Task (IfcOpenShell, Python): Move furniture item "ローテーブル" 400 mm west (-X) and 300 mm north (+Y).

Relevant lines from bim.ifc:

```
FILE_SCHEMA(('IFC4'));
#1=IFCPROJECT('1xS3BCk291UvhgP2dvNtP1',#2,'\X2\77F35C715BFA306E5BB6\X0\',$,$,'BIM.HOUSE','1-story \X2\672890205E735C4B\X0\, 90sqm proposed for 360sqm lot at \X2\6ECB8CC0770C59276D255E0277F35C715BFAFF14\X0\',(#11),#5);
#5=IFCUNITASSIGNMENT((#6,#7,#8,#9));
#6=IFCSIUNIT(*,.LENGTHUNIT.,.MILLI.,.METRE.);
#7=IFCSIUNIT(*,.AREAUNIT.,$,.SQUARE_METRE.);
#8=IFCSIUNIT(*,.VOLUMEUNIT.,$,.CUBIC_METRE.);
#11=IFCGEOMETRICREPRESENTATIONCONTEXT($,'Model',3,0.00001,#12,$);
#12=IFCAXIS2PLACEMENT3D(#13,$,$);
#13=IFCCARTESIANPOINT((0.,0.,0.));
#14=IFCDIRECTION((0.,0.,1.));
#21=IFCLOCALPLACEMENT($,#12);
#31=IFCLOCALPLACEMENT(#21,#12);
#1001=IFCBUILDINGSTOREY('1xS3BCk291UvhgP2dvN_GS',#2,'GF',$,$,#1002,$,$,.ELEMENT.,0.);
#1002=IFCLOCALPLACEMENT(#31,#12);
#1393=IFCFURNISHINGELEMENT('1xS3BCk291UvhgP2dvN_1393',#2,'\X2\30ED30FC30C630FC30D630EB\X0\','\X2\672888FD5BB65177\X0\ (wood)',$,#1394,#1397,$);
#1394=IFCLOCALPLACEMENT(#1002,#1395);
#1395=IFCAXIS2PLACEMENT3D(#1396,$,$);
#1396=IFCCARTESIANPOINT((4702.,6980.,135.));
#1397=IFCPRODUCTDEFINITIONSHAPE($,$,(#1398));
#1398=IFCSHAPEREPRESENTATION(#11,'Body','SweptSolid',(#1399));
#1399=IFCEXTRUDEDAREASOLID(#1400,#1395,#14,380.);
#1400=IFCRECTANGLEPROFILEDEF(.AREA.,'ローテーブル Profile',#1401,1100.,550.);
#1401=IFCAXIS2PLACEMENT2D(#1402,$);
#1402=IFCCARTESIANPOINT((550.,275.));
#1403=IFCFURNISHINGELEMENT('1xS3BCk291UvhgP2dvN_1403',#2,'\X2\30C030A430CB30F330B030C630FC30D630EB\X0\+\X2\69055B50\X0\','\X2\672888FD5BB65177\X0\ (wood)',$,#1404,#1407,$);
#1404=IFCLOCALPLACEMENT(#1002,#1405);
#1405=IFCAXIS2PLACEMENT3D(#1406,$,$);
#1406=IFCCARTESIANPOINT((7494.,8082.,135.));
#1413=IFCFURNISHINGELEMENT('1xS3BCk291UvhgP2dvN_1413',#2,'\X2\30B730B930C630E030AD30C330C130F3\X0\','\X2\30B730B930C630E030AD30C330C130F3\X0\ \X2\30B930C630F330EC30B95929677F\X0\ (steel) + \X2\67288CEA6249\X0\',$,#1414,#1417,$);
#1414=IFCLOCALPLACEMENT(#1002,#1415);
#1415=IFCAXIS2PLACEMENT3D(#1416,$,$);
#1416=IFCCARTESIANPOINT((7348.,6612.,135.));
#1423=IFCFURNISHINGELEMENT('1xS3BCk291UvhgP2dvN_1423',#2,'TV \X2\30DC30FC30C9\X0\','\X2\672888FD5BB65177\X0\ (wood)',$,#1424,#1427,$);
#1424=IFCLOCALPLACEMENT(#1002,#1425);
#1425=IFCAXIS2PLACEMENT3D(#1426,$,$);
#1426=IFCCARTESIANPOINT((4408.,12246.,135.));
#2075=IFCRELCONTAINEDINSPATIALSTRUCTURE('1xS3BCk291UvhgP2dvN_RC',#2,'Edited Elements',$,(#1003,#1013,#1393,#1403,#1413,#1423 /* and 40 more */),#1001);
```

```python
import ifcopenshell
import ifcopenshell.api.geometry
import ifcopenshell.util.placement

model = ifcopenshell.open("bim.ifc")

item = model.by_guid("1xS3BCk291UvhgP2dvN_1393")
matrix = ifcopenshell.util.placement.get_local_placement(item.ObjectPlacement)
matrix[0, 3] -= 400.0
matrix[1, 3] += 300.0
ifcopenshell.api.geometry.edit_object_placement(model, product=item, matrix=matrix, is_si=False)

print(ifcopenshell.util.placement.get_local_placement(item.ObjectPlacement).round(3) + 0.0)

model.write("bim_v2.ifc")
```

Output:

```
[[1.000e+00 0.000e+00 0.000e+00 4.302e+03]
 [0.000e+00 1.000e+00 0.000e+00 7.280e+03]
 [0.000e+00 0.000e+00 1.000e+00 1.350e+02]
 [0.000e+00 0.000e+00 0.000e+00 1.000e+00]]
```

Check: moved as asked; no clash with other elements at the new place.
